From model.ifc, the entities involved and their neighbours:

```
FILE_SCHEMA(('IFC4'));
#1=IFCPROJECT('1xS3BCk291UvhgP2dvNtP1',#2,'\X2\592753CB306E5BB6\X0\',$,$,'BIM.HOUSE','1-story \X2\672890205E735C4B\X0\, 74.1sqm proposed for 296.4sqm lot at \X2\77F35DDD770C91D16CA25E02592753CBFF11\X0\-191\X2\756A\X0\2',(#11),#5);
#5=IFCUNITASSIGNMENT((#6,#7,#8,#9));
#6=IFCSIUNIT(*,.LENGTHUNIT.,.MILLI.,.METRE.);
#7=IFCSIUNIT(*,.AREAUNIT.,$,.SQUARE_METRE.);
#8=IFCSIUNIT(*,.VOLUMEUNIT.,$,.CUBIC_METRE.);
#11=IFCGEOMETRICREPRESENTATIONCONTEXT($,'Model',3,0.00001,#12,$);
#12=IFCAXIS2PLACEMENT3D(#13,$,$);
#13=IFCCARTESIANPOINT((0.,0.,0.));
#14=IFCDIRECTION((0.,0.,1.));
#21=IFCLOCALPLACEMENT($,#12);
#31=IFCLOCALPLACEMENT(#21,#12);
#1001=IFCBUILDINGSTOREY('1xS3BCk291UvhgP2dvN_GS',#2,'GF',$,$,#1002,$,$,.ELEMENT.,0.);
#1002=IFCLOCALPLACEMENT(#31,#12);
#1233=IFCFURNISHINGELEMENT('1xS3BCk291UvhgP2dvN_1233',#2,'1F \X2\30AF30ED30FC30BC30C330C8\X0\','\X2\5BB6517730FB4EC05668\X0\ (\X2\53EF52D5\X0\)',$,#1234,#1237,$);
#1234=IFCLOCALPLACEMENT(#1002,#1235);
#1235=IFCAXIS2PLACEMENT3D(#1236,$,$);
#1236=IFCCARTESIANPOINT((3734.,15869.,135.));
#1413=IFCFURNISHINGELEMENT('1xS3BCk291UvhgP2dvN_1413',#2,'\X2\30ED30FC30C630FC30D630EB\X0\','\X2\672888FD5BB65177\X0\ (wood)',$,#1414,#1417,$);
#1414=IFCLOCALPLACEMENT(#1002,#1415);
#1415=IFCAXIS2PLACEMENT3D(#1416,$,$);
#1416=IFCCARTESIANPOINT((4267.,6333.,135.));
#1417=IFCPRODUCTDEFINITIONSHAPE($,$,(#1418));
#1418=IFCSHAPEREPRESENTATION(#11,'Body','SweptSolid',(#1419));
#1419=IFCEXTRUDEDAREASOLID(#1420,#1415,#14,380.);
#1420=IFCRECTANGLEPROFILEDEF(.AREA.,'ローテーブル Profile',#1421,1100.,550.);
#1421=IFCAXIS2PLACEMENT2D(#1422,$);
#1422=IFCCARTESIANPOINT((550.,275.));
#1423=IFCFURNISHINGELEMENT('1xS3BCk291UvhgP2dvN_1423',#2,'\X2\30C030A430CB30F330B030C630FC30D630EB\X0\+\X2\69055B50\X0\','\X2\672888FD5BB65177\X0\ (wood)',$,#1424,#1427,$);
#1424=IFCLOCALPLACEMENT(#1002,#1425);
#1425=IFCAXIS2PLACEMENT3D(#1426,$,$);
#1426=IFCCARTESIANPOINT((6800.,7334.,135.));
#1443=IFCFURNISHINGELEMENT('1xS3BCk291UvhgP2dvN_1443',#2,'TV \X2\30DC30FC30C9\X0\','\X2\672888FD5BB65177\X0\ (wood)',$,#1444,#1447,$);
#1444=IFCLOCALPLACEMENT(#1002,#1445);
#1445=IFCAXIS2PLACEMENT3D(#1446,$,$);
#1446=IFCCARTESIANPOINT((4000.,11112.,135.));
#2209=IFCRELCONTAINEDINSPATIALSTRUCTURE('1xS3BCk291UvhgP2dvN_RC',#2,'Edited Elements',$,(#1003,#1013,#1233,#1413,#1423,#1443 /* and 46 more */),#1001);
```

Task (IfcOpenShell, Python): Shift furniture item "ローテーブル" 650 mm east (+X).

```python
import ifcopenshell
import ifcopenshell.api.geometry
import ifcopenshell.util.placement
import ifcopenshell.util.unit

model = ifcopenshell.open("model.ifc")
unit_scale = ifcopenshell.util.unit.calculate_unit_scale(model)

item = model.by_guid("1xS3BCk291UvhgP2dvN_1413")
matrix = ifcopenshell.util.placement.get_local_placement(item.ObjectPlacement)
matrix[0, 3] += 0.65 / unit_scale
ifcopenshell.api.geometry.edit_object_placement(model, product=item, matrix=matrix, is_si=False)

print(ifcopenshell.util.placement.get_local_placement(item.ObjectPlacement).round(3) + 0.0)

model.write("model_updated.ifc")
```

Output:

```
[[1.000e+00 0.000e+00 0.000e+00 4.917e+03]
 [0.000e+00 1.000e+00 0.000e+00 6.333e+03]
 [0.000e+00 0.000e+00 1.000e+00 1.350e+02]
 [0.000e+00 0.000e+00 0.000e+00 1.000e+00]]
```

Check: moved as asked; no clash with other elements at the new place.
